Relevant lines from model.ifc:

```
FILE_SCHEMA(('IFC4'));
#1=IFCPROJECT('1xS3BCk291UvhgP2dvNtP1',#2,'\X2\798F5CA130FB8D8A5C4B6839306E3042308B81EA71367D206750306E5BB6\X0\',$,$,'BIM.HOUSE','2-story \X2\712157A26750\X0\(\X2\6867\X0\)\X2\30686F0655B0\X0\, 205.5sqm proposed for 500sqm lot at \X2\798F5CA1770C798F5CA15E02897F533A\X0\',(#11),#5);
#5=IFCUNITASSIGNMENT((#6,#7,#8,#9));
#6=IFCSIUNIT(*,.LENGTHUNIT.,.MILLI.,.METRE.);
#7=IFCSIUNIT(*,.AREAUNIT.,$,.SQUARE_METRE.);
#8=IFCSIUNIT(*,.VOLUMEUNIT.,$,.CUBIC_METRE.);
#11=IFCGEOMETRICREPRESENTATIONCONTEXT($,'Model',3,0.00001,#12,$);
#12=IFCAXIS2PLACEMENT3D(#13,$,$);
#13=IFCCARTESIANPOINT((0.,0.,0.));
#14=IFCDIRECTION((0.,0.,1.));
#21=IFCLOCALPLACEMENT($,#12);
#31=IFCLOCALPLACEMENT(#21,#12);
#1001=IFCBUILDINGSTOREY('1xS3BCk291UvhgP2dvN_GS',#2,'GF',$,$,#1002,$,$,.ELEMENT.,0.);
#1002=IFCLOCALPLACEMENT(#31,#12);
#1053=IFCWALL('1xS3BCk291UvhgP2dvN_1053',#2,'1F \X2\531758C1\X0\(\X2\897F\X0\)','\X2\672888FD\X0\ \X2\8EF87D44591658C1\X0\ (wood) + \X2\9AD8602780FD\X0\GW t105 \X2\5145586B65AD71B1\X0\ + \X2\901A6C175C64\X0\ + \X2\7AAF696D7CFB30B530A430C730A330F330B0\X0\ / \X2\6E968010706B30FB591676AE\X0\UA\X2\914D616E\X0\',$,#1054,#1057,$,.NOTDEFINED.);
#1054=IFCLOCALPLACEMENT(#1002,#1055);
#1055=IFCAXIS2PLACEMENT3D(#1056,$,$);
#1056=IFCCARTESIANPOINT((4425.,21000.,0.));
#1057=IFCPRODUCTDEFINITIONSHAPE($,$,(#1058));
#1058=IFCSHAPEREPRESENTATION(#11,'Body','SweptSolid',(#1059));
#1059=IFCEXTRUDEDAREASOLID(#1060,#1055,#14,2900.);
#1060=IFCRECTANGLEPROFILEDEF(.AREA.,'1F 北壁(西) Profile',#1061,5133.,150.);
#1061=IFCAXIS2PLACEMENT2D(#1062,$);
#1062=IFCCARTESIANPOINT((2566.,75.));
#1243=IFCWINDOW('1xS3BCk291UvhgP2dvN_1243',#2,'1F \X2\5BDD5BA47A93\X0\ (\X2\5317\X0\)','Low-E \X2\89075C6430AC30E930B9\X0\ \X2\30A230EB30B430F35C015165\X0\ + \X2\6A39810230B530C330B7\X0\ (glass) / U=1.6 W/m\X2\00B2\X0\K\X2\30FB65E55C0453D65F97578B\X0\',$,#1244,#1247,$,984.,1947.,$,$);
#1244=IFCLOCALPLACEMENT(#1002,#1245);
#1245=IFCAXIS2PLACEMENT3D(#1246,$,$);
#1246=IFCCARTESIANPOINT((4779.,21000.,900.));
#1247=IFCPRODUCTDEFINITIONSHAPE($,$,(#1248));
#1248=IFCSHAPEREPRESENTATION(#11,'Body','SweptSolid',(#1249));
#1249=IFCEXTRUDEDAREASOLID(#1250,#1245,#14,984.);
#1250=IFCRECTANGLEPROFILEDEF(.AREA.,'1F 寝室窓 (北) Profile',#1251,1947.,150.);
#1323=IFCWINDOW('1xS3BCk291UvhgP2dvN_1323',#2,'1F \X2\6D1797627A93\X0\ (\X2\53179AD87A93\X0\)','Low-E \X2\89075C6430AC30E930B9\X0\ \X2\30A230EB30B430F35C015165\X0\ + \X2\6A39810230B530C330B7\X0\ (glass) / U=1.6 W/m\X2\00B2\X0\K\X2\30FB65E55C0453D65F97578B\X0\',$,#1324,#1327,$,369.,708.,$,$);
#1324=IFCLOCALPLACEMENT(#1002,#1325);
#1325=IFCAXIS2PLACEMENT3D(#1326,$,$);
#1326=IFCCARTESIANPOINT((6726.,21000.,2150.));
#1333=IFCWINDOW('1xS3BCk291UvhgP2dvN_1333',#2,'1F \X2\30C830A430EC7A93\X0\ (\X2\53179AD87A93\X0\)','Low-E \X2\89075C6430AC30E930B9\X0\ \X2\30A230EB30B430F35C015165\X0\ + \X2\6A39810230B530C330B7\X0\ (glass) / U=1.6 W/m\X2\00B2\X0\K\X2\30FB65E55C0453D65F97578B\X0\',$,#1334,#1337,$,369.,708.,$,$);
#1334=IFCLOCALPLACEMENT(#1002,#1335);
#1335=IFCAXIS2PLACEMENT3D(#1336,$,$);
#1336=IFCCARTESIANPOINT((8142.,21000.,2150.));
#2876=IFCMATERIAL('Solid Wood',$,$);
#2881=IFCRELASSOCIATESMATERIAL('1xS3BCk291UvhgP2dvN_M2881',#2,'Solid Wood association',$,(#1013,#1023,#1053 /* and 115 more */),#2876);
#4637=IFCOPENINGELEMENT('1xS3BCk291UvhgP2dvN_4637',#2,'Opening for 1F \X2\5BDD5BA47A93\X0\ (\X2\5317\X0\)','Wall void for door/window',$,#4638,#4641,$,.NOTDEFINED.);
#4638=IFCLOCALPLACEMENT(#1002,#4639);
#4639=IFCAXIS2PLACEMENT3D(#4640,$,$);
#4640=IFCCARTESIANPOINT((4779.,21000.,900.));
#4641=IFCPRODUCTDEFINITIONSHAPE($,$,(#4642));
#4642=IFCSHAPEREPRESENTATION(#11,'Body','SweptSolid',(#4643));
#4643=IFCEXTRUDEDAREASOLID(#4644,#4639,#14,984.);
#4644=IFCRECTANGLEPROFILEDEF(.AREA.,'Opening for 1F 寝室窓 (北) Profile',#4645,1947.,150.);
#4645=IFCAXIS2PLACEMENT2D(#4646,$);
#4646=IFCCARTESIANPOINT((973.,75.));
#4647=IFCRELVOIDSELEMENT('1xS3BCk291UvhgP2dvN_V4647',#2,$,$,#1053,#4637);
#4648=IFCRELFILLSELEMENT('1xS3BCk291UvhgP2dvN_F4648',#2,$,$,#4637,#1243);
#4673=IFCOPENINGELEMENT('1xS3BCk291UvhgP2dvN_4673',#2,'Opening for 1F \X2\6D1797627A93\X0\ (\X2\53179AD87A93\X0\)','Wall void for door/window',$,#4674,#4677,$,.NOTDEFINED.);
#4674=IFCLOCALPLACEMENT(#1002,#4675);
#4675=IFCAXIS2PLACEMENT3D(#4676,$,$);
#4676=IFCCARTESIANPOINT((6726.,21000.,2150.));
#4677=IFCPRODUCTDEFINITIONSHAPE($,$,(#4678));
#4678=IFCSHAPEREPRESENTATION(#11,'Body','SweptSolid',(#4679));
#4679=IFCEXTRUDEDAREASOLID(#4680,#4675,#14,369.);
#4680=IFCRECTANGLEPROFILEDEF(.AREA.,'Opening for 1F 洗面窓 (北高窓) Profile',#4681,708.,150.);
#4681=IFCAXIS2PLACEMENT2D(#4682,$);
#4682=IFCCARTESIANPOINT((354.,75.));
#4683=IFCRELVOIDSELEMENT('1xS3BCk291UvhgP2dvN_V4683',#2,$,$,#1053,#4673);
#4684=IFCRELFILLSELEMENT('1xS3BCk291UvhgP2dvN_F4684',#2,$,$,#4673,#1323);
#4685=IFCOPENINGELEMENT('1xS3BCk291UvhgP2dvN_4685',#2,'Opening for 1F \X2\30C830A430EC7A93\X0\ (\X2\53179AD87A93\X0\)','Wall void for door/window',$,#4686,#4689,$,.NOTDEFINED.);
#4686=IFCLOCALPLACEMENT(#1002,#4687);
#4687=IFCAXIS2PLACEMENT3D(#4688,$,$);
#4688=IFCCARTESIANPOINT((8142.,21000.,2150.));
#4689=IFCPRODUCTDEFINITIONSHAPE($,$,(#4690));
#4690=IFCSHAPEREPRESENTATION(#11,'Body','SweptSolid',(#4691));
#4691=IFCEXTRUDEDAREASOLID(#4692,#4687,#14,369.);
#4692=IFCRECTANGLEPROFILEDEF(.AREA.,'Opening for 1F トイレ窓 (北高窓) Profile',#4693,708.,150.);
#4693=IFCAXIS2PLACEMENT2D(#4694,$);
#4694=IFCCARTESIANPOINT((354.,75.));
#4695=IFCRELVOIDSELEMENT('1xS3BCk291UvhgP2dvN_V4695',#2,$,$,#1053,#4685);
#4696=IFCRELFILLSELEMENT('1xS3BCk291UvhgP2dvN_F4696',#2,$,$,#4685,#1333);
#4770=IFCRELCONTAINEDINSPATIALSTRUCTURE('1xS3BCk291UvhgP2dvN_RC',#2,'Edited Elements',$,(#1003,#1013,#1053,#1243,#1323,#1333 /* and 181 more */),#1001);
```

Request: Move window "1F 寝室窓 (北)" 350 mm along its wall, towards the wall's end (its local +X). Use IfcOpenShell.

```python
import ifcopenshell
import ifcopenshell.api.geometry
import ifcopenshell.util.placement
import ifcopenshell.util.unit

model = ifcopenshell.open("model.ifc")
unit_scale = ifcopenshell.util.unit.calculate_unit_scale(model)

window = model.by_guid("1xS3BCk291UvhgP2dvN_1243")
opening = window.FillsVoids[0].RelatingOpeningElement
wall = opening.VoidsElements[0].RelatingBuildingElement

wall_matrix = ifcopenshell.util.placement.get_local_placement(wall.ObjectPlacement)
shift = wall_matrix[:3, 0] * 0.35 / unit_scale
before = ifcopenshell.util.placement.get_local_placement(window.ObjectPlacement)[:3, 3].copy()

# The window is not placed relative to its opening, so move both.
for product in (opening, window):
    matrix = ifcopenshell.util.placement.get_local_placement(product.ObjectPlacement)
    matrix[:3, 3] += shift
    ifcopenshell.api.geometry.edit_object_placement(model, product=product, matrix=matrix, is_si=False)

after = ifcopenshell.util.placement.get_local_placement(window.ObjectPlacement)[:3, 3]
print("window moved by", (after - before).round(3) + 0.0)

model.write("model_v2.ifc")
```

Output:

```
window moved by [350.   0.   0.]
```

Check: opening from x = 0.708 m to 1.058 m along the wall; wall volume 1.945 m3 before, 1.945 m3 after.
